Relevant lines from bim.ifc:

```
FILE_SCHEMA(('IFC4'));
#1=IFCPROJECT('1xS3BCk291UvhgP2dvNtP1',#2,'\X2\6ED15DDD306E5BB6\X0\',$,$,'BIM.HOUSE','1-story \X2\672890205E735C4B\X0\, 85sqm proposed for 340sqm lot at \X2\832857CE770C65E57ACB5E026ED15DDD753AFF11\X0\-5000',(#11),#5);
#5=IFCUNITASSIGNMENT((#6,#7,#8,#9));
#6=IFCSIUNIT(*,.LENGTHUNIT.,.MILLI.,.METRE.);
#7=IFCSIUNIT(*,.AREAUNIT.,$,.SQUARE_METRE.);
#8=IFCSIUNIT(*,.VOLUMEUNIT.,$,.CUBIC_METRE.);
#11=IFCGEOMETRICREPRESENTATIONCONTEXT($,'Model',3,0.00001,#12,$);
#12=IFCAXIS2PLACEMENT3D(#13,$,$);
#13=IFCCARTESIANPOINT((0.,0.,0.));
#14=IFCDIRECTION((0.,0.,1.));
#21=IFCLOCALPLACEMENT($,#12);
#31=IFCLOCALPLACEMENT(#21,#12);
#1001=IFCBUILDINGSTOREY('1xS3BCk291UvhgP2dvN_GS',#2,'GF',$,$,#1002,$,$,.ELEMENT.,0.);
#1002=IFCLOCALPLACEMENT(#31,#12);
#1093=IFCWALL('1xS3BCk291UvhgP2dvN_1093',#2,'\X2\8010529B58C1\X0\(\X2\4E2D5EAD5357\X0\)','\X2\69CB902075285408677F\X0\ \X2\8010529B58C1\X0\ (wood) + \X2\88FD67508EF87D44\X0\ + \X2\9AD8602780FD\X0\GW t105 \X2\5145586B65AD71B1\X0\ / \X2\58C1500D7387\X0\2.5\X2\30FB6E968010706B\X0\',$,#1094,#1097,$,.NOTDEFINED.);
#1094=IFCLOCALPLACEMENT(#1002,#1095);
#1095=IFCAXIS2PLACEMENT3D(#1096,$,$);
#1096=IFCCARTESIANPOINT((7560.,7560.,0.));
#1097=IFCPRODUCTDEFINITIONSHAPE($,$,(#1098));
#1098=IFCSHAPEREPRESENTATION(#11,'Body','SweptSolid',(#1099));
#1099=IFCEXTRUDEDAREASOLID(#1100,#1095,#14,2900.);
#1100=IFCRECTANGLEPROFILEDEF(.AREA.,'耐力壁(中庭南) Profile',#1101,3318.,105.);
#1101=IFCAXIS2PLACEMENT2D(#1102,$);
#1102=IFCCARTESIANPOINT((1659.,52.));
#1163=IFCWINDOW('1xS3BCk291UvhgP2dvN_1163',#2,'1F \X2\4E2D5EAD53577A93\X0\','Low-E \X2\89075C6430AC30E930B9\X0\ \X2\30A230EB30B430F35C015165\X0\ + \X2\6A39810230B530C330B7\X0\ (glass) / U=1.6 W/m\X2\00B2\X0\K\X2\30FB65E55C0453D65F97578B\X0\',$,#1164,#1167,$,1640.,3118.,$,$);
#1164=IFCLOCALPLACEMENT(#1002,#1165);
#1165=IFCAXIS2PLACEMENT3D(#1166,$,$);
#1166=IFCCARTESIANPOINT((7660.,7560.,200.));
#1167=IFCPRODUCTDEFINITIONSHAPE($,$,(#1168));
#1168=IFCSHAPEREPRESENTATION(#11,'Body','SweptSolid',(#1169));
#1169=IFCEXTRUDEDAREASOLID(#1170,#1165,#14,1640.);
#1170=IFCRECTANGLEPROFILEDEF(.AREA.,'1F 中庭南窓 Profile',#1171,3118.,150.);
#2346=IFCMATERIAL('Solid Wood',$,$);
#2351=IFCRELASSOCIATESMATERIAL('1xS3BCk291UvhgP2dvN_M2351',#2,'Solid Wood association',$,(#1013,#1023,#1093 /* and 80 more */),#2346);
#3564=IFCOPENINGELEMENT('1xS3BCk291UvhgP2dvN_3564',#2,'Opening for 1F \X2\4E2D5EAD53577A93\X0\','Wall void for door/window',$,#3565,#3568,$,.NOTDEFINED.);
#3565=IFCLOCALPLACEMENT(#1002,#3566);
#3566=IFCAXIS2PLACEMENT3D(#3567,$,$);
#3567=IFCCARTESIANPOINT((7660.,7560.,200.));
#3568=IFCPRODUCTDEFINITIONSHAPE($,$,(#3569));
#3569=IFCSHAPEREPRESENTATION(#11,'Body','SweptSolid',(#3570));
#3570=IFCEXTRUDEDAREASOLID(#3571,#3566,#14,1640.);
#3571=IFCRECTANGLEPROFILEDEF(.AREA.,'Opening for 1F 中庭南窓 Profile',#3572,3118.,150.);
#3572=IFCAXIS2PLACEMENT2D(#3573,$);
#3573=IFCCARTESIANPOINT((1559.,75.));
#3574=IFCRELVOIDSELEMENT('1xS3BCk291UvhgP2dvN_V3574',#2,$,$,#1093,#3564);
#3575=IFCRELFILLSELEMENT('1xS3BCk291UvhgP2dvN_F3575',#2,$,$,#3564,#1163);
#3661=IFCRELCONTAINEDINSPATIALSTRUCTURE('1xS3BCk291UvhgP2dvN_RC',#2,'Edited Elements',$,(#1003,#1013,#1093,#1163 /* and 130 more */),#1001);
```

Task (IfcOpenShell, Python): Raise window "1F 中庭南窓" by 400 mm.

```python
import numpy as np
import ifcopenshell
import ifcopenshell.api.geometry
import ifcopenshell.util.placement
import ifcopenshell.util.unit

model = ifcopenshell.open("bim.ifc")
unit_scale = ifcopenshell.util.unit.calculate_unit_scale(model)

window = model.by_id(1163)
opening = window.FillsVoids[0].RelatingOpeningElement
dz = 400.0

shift = np.array([0.0, 0.0, dz])
# The window is not placed relative to its opening, so move both.
for product in (opening, window):
    matrix = ifcopenshell.util.placement.get_local_placement(product.ObjectPlacement)
    matrix[:3, 3] += shift
    ifcopenshell.api.geometry.edit_object_placement(model, product=product, matrix=matrix, is_si=False)

print(f"moved by {dz * unit_scale:+.3f} m")

model.write("bim_v2.ifc")
```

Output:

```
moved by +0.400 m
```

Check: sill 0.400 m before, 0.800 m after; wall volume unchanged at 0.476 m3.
